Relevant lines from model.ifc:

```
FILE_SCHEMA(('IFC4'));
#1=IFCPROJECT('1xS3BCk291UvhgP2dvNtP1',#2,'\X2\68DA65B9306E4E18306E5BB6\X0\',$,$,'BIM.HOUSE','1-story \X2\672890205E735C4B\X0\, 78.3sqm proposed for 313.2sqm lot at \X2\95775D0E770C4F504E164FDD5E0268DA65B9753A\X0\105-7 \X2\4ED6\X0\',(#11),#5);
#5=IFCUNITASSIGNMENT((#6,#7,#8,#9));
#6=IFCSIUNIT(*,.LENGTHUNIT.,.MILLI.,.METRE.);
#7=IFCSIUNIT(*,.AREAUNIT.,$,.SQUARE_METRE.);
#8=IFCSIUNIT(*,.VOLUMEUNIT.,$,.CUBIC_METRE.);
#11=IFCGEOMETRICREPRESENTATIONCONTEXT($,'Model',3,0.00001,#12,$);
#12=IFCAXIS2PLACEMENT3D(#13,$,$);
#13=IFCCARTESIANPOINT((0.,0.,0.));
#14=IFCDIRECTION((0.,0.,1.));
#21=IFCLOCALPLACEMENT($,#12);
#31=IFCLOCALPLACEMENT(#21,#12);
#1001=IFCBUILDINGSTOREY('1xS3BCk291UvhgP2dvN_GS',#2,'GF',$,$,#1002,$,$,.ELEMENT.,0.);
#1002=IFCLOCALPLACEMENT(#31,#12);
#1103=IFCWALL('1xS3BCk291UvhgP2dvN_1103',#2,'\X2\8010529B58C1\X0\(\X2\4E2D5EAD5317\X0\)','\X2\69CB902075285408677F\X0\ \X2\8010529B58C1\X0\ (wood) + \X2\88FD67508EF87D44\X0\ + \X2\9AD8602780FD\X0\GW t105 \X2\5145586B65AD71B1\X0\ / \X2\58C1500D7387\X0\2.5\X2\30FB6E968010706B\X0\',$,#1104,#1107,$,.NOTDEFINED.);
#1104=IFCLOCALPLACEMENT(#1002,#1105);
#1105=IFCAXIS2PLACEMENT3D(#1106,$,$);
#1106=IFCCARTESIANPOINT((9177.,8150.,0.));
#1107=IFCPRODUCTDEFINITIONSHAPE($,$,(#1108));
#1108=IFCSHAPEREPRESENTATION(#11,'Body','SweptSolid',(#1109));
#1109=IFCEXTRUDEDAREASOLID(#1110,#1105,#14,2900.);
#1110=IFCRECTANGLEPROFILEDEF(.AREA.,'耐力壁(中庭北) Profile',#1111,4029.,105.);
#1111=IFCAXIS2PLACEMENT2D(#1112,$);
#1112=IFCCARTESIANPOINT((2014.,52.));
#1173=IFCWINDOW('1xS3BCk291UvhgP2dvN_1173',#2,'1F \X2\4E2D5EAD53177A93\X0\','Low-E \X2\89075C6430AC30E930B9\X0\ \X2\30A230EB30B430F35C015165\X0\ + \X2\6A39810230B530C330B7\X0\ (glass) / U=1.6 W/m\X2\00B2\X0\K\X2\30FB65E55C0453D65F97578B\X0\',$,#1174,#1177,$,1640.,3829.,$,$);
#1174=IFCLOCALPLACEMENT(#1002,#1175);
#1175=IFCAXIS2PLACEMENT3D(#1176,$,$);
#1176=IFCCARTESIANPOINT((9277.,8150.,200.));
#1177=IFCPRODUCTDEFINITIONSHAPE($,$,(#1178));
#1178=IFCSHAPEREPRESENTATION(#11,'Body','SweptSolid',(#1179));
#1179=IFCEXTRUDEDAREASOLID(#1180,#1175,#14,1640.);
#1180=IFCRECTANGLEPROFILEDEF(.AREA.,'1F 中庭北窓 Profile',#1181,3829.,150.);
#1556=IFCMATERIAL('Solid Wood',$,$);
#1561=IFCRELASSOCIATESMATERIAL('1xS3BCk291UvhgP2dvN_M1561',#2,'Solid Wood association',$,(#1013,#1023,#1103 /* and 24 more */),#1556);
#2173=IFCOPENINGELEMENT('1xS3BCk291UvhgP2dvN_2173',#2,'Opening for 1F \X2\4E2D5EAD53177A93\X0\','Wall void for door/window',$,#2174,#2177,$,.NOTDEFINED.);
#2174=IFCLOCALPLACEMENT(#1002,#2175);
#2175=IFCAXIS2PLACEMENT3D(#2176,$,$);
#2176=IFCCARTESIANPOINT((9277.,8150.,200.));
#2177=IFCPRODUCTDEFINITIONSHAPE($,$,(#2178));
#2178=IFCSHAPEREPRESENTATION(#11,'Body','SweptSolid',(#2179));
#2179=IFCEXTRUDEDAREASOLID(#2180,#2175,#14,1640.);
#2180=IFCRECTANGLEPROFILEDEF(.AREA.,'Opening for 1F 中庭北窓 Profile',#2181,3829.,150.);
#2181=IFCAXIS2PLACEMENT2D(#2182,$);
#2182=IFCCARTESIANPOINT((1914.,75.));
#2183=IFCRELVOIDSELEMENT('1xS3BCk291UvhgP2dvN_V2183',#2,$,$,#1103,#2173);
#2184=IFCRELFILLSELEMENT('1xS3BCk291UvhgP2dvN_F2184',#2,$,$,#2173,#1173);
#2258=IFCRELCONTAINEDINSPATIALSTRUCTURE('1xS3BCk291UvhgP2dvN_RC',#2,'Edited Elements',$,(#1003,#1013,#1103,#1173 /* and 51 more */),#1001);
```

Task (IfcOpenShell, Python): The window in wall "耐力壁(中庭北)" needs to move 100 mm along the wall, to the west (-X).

```python
import ifcopenshell
import ifcopenshell.api.geometry
import ifcopenshell.util.placement
import ifcopenshell.util.unit

model = ifcopenshell.open("model.ifc")
unit_scale = ifcopenshell.util.unit.calculate_unit_scale(model)

window = model.by_guid("1xS3BCk291UvhgP2dvN_1173")
opening = window.FillsVoids[0].RelatingOpeningElement
wall = opening.VoidsElements[0].RelatingBuildingElement

wall_matrix = ifcopenshell.util.placement.get_local_placement(wall.ObjectPlacement)
shift = wall_matrix[:3, 0] * -0.1 / unit_scale
before = ifcopenshell.util.placement.get_local_placement(window.ObjectPlacement)[:3, 3].copy()

# The window is not placed relative to its opening, so move both.
for product in (opening, window):
    matrix = ifcopenshell.util.placement.get_local_placement(product.ObjectPlacement)
    matrix[:3, 3] += shift
    ifcopenshell.api.geometry.edit_object_placement(model, product=product, matrix=matrix, is_si=False)

after = ifcopenshell.util.placement.get_local_placement(window.ObjectPlacement)[:3, 3]
print("window moved by", (after - before).round(3) + 0.0)

model.write("model_updated.ifc")
```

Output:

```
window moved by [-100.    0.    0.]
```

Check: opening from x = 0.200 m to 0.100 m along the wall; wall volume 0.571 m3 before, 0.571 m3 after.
